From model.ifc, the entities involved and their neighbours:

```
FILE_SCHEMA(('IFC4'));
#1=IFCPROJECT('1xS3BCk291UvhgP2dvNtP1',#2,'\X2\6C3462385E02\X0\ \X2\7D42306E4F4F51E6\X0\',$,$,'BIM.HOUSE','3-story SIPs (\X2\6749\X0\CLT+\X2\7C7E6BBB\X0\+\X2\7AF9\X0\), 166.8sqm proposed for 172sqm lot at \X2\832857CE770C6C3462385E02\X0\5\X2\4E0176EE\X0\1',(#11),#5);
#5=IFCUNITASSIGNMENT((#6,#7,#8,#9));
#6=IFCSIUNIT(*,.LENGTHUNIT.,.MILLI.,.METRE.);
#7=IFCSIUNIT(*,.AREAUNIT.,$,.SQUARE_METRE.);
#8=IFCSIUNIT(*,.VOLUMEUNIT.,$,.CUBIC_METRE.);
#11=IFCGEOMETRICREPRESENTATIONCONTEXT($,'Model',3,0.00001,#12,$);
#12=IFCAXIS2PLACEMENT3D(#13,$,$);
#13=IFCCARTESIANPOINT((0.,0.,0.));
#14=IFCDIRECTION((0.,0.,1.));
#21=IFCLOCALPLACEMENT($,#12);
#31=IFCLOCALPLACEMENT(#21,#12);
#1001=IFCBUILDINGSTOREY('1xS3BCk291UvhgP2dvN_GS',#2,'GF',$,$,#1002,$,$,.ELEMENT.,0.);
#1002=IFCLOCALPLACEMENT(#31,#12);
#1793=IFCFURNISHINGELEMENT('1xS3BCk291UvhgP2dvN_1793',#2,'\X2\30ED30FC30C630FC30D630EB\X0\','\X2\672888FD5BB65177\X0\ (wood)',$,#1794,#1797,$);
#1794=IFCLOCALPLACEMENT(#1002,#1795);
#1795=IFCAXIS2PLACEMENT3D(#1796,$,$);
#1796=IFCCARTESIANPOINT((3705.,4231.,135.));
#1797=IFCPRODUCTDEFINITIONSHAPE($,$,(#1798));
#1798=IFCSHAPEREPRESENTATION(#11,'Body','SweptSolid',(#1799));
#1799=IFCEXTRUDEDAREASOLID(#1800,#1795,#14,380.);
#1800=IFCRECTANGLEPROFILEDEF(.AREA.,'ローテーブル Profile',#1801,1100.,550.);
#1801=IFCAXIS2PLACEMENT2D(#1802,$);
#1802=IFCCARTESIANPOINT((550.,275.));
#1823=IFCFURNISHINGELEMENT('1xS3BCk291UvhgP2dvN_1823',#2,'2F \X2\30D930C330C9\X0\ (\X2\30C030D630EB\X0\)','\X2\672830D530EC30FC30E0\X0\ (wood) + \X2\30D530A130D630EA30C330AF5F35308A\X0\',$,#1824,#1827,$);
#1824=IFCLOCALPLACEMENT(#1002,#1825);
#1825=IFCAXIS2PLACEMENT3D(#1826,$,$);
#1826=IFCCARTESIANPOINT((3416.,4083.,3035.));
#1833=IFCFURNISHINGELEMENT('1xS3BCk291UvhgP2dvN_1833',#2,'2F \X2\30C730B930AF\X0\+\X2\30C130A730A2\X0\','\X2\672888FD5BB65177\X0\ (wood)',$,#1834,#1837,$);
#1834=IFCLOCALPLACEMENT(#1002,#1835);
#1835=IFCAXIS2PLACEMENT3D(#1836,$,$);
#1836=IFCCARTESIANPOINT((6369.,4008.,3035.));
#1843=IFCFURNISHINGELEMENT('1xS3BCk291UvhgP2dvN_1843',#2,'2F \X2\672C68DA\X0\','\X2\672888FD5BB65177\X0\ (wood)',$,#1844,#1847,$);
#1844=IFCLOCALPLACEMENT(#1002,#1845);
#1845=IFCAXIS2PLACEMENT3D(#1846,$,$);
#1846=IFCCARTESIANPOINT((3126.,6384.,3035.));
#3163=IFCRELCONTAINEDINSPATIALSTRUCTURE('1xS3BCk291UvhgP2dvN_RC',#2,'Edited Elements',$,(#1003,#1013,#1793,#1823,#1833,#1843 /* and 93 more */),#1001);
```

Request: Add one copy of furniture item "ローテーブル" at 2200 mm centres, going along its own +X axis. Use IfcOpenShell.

```python
import ifcopenshell
import ifcopenshell.api.geometry
import ifcopenshell.api.root
import ifcopenshell.util.element
import ifcopenshell.util.placement
import ifcopenshell.util.unit

model = ifcopenshell.open("model.ifc")
unit_scale = ifcopenshell.util.unit.calculate_unit_scale(model)


def reuse_history(source, copy):
    """copy_class also copies each property set's owner history, people and application; keep the originals."""
    for rel in copy.IsDefinedBy:
        if rel.is_a("IfcRelDefinesByProperties") and (history := rel.RelatingPropertyDefinition.OwnerHistory):
            rel.RelatingPropertyDefinition.OwnerHistory = source.OwnerHistory
            ifcopenshell.util.element.remove_deep2(model, history)


source = model.by_id(1793)
base = ifcopenshell.util.placement.get_local_placement(source.ObjectPlacement)
step = base[:3, 0] * 2.2 / unit_scale

for i in range(1, 2):
    copy = ifcopenshell.api.root.copy_class(model, product=source)
    copy.Representation = ifcopenshell.util.element.copy_deep(
        model, source.Representation, exclude=["IfcGeometricRepresentationContext", "IfcRepresentationMap"]
    )
    reuse_history(source, copy)
    matrix = base.copy()
    matrix[:3, 3] += i * step
    print("added at", matrix[:3, 3].round(3) + 0.0)
    ifcopenshell.api.geometry.edit_object_placement(model, product=copy, matrix=matrix, is_si=False)

model.write("model_v2.ifc")
```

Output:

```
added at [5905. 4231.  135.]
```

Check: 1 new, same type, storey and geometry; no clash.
